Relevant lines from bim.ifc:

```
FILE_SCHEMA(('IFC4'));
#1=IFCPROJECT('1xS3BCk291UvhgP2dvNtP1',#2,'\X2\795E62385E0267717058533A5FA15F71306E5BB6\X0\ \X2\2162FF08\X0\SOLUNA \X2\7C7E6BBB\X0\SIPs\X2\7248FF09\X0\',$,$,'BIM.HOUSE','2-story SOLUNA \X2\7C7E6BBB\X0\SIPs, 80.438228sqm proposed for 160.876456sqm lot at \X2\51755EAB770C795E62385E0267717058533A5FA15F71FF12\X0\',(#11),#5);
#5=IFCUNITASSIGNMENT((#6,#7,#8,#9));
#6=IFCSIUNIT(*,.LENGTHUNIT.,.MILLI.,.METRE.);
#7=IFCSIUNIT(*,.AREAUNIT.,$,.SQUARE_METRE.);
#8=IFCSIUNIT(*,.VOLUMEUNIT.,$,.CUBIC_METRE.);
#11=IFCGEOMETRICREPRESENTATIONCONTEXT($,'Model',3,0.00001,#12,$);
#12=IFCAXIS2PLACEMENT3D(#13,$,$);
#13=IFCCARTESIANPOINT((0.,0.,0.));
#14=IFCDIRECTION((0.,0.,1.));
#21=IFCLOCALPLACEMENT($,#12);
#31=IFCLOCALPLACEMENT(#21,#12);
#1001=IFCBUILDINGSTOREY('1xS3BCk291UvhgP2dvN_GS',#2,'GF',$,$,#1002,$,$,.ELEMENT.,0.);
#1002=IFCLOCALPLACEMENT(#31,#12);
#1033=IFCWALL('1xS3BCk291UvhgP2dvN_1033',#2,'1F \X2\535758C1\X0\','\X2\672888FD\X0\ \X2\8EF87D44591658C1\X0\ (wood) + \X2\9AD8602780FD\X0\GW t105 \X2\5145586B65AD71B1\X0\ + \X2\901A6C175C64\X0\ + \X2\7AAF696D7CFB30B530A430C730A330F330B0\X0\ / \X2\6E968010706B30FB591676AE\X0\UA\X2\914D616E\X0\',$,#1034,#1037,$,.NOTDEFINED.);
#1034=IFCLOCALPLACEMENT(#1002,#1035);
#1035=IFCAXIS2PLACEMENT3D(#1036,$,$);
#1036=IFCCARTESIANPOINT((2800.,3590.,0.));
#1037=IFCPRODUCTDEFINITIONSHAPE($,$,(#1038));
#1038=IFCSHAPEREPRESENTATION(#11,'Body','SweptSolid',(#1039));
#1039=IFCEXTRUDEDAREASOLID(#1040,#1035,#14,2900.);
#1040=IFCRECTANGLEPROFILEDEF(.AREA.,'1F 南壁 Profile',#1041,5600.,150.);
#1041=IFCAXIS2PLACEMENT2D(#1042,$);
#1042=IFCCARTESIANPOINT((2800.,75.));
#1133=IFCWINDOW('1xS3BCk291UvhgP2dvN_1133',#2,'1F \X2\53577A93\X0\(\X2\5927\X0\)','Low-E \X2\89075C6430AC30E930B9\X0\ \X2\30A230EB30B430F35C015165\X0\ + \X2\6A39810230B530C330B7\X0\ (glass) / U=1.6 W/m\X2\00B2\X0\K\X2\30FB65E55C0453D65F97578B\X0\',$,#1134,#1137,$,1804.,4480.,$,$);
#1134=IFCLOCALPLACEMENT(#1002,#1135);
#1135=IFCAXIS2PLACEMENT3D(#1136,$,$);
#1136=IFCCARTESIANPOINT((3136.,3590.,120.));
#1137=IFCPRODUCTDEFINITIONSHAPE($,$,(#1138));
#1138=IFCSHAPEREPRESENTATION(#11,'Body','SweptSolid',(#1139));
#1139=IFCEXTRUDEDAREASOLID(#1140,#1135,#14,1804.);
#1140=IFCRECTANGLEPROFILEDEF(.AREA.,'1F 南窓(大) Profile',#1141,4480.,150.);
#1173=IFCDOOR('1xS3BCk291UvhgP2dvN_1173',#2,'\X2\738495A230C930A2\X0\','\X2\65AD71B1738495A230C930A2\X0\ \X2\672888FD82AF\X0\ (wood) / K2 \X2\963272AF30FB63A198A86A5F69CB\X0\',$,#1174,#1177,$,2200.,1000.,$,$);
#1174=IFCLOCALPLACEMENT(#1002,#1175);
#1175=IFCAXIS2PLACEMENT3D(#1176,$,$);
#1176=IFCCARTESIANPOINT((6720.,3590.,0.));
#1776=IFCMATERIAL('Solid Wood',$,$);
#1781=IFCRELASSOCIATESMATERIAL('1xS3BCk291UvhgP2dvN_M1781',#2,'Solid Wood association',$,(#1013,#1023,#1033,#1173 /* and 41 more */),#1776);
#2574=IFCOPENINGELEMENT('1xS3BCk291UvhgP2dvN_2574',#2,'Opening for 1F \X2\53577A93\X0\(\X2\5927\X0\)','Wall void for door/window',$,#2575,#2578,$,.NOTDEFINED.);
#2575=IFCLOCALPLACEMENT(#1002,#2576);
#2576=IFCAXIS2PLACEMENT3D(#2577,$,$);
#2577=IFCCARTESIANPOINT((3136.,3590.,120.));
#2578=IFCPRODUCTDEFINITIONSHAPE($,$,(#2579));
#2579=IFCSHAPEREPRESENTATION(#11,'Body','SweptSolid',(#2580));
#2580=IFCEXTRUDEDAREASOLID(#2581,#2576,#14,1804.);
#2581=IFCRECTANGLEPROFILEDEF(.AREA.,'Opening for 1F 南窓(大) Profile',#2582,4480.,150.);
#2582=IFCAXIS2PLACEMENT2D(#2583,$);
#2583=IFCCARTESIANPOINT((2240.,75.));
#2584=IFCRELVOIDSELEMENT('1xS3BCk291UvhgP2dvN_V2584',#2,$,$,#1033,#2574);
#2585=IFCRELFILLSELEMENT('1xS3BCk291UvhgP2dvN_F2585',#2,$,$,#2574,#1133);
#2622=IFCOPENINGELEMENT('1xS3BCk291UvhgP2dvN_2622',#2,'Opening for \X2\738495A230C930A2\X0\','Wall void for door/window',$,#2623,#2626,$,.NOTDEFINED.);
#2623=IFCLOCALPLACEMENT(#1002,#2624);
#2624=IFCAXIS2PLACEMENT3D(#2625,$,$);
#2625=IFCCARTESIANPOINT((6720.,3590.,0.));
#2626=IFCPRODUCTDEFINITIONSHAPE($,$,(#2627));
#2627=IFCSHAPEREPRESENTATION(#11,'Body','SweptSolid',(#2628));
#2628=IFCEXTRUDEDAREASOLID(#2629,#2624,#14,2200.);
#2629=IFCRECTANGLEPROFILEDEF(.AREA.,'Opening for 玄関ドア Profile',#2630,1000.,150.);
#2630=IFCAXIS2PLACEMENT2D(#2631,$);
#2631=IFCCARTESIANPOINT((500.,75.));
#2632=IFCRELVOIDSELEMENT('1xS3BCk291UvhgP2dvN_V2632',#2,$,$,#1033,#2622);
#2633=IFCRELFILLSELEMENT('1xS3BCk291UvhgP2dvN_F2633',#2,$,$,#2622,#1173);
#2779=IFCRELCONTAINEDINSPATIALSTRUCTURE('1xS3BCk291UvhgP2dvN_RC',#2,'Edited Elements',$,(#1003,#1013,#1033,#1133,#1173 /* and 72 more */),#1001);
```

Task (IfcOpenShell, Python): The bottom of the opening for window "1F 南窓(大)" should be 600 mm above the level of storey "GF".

```python
import numpy as np
import ifcopenshell
import ifcopenshell.api.geometry
import ifcopenshell.geom
import ifcopenshell.util.element
import ifcopenshell.util.placement
import ifcopenshell.util.shape
import ifcopenshell.util.unit

model = ifcopenshell.open("bim.ifc")
unit_scale = ifcopenshell.util.unit.calculate_unit_scale(model)

window = model.by_guid("1xS3BCk291UvhgP2dvN_1133")
opening = window.FillsVoids[0].RelatingOpeningElement
storey = ifcopenshell.util.element.get_container(window, ifc_class="IfcBuildingStorey")
level = ifcopenshell.util.placement.get_local_placement(storey.ObjectPlacement)[2, 3]

# The opening's origin need not be at the sill, so measure its lowest point.
shape = ifcopenshell.geom.create_shape(ifcopenshell.geom.settings(), opening)
bottom = ifcopenshell.util.shape.get_shape_bottom_elevation(shape, shape.geometry) / unit_scale
dz = level + 0.6 / unit_scale - bottom

shift = np.array([0.0, 0.0, dz])
# The window is not placed relative to its opening, so move both.
for product in (opening, window):
    matrix = ifcopenshell.util.placement.get_local_placement(product.ObjectPlacement)
    matrix[:3, 3] += shift
    ifcopenshell.api.geometry.edit_object_placement(model, product=product, matrix=matrix, is_si=False)

print(f"moved by {dz * unit_scale:+.3f} m")

model.write("bim_rev.ifc")
```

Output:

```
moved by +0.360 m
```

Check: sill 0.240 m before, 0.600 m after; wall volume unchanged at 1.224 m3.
